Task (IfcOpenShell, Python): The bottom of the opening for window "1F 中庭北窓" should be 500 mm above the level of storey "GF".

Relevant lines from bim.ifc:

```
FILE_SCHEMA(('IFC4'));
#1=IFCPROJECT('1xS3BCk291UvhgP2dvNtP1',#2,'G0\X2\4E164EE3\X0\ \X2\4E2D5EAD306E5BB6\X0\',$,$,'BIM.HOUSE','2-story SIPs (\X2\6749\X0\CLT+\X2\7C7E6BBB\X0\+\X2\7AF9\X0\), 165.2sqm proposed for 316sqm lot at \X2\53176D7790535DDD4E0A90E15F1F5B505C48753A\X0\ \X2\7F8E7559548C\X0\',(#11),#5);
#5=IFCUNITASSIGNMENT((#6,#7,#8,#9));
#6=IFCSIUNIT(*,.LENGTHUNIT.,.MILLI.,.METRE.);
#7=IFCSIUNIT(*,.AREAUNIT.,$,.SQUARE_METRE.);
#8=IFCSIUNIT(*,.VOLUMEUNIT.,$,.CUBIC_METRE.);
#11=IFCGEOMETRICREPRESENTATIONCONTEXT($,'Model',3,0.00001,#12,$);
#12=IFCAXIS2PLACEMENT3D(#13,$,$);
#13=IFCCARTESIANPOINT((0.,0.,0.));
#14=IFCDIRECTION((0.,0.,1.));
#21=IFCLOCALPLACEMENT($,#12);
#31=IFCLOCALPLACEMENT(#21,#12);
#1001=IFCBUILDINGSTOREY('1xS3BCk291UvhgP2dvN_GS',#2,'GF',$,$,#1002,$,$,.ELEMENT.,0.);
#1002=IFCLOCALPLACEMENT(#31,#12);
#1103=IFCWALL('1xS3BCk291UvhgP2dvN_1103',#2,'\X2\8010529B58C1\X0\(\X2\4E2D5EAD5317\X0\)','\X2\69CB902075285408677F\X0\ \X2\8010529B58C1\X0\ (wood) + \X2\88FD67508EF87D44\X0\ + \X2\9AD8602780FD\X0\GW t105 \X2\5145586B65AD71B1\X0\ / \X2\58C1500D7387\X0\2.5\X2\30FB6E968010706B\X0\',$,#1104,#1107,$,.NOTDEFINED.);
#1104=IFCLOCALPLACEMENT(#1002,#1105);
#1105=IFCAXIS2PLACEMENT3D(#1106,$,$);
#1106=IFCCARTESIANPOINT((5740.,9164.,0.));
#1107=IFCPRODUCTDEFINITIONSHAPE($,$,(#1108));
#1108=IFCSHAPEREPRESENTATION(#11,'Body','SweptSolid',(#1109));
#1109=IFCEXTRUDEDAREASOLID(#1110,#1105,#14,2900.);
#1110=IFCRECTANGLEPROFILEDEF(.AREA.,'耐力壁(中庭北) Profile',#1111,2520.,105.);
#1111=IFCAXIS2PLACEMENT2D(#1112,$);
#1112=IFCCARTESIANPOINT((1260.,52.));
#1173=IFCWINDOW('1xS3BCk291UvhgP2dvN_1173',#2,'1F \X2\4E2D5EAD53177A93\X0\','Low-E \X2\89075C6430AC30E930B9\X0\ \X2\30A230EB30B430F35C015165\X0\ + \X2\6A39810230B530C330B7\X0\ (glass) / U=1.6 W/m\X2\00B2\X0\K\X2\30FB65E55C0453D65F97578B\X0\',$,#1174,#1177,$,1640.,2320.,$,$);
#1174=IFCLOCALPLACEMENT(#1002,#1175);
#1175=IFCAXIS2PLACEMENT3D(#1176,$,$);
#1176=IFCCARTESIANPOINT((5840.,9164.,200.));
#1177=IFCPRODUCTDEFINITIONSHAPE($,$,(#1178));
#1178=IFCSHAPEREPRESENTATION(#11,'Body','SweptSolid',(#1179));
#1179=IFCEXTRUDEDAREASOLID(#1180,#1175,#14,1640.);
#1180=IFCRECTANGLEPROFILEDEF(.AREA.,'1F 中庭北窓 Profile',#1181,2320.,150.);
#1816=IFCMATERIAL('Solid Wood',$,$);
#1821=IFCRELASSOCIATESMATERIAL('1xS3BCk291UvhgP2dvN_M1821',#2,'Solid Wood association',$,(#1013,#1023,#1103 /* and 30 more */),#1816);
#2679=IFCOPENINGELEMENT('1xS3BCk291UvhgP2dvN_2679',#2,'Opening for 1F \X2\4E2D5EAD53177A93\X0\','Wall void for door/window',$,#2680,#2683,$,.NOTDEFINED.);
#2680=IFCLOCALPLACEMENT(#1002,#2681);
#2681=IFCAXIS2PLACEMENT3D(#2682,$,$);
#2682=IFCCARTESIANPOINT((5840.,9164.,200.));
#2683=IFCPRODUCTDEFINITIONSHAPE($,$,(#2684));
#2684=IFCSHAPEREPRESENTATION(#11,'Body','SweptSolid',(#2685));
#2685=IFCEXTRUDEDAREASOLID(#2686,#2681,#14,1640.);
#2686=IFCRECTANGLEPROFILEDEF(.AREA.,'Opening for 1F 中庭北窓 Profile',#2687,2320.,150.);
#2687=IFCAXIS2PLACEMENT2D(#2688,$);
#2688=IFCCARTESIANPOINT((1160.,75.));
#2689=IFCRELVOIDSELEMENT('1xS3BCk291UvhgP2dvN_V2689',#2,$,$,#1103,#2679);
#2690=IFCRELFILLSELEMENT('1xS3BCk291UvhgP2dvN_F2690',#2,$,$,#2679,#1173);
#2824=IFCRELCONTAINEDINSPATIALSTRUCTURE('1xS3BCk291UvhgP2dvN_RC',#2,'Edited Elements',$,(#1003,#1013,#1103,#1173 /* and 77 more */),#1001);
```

```python
import numpy as np
import ifcopenshell
import ifcopenshell.api.geometry
import ifcopenshell.geom
import ifcopenshell.util.element
import ifcopenshell.util.placement
import ifcopenshell.util.shape
import ifcopenshell.util.unit

model = ifcopenshell.open("bim.ifc")
unit_scale = ifcopenshell.util.unit.calculate_unit_scale(model)

window = model.by_guid("1xS3BCk291UvhgP2dvN_1173")
opening = window.FillsVoids[0].RelatingOpeningElement
storey = ifcopenshell.util.element.get_container(window, ifc_class="IfcBuildingStorey")
level = ifcopenshell.util.placement.get_local_placement(storey.ObjectPlacement)[2, 3]

# The opening's origin need not be at the sill, so measure its lowest point.
shape = ifcopenshell.geom.create_shape(ifcopenshell.geom.settings(), opening)
bottom = ifcopenshell.util.shape.get_shape_bottom_elevation(shape, shape.geometry) / unit_scale
dz = level + 500.0 - bottom

shift = np.array([0.0, 0.0, dz])
# The window is not placed relative to its opening, so move both.
for product in (opening, window):
    matrix = ifcopenshell.util.placement.get_local_placement(product.ObjectPlacement)
    matrix[:3, 3] += shift
    ifcopenshell.api.geometry.edit_object_placement(model, product=product, matrix=matrix, is_si=False)

print(f"moved by {dz * unit_scale:+.3f} m")

model.write("bim_v2.ifc")
```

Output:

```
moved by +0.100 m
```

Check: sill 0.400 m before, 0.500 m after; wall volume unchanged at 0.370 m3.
